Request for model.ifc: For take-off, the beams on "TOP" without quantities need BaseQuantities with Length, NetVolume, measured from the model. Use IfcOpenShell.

First a look at what the model holds.

```python
import ifcopenshell
import ifcopenshell.util.element
import ifcopenshell.util.unit

model = ifcopenshell.open("model.ifc")
print(model.schema)
for unit_type in ("LENGTHUNIT", "AREAUNIT", "VOLUMEUNIT"):
    print(unit_type, ifcopenshell.util.unit.calculate_unit_scale(model, unit_type))
storey = next(s for s in model.by_type("IfcBuildingStorey") if s.Name == "TOP")
beams = [e for e in ifcopenshell.util.element.get_decomposition(storey) if e.is_a("IfcBeam")]
for e in sorted(beams, key=lambda e: e.id()):
    print(e.id(), e.is_a(), e.Name, list(ifcopenshell.util.element.get_psets(e, qtos_only=True)), sep=" | ")
```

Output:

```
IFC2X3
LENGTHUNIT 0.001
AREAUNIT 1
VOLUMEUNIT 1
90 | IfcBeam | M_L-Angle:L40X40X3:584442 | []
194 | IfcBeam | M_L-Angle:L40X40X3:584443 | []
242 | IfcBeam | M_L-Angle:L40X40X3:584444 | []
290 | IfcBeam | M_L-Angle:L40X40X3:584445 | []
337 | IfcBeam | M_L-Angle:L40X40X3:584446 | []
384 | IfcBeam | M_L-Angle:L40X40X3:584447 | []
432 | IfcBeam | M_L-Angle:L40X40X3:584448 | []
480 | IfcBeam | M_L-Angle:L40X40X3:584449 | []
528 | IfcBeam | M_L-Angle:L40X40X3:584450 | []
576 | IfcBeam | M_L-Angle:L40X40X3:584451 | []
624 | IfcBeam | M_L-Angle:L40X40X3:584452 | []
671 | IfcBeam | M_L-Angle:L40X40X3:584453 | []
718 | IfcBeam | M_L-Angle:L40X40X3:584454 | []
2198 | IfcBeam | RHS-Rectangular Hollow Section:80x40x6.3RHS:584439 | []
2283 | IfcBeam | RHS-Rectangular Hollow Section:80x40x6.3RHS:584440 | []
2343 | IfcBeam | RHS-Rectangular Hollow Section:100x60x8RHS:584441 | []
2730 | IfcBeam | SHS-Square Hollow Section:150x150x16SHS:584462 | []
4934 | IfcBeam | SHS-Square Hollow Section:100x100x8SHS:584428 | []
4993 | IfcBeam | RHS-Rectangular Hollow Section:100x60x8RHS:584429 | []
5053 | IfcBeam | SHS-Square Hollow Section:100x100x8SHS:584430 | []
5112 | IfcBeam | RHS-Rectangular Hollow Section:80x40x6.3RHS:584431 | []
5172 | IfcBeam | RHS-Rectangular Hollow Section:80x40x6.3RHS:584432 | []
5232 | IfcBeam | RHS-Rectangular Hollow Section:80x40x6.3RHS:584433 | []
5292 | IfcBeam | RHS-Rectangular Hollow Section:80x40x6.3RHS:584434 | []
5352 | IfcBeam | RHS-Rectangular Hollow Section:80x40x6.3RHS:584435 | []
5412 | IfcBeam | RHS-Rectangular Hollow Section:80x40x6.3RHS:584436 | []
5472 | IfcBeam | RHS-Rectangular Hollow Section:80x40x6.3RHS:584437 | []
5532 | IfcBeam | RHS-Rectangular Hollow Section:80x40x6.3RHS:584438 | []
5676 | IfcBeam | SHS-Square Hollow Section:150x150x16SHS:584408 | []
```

```python
import ifcopenshell
import ifcopenshell.api.pset
import ifcopenshell.geom
import ifcopenshell.util.element
import ifcopenshell.util.shape
import ifcopenshell.util.unit

model = ifcopenshell.open("model.ifc")
unit_scale = ifcopenshell.util.unit.calculate_unit_scale(model)
volume_scale = ifcopenshell.util.unit.calculate_unit_scale(model, "VOLUMEUNIT")
settings = ifcopenshell.geom.settings()

storey = next(s for s in model.by_type("IfcBuildingStorey") if s.Name == "TOP")
beams = [e for e in ifcopenshell.util.element.get_decomposition(storey) if e.is_a("IfcBeam")]

for e in sorted(beams, key=lambda e: e.id()):
    if ifcopenshell.util.element.get_psets(e, qtos_only=True, should_inherit=False):
        continue
    # Geometry comes back in metres, in the element's own axes.
    shape = ifcopenshell.geom.create_shape(settings, e)
    values = {
        "Length": ifcopenshell.util.shape.get_max_xyz(shape.geometry) / unit_scale,
        "NetVolume": ifcopenshell.util.shape.get_volume(shape.geometry) / volume_scale,
    }
    qto = ifcopenshell.api.pset.add_qto(model, product=e, name="BaseQuantities")
    ifcopenshell.api.pset.edit_qto(model, qto=qto, properties=values)
    print(e.id(), {k: round(v, 3) for k, v in values.items()})

model.write("model_edited.ifc")
```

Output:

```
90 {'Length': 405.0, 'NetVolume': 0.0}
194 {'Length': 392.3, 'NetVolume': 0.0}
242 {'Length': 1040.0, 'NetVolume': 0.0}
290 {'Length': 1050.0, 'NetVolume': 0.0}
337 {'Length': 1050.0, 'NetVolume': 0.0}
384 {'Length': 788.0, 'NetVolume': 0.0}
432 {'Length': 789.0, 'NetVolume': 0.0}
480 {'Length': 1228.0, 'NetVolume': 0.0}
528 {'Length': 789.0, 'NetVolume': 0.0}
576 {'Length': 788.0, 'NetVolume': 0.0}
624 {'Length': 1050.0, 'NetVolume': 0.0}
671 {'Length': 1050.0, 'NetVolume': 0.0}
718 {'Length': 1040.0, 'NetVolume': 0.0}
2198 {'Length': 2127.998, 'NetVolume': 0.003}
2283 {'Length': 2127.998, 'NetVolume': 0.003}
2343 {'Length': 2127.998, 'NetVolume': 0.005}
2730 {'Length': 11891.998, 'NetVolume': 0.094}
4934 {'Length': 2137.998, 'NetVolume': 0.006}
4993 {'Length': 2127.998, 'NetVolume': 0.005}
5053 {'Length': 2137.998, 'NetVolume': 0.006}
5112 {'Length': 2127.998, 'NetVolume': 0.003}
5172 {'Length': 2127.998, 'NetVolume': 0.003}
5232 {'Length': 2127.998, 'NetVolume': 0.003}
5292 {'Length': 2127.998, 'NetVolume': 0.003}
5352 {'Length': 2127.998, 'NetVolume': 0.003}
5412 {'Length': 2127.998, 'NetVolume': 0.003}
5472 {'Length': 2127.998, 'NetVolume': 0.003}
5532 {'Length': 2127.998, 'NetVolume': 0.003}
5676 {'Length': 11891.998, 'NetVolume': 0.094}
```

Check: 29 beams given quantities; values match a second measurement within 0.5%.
